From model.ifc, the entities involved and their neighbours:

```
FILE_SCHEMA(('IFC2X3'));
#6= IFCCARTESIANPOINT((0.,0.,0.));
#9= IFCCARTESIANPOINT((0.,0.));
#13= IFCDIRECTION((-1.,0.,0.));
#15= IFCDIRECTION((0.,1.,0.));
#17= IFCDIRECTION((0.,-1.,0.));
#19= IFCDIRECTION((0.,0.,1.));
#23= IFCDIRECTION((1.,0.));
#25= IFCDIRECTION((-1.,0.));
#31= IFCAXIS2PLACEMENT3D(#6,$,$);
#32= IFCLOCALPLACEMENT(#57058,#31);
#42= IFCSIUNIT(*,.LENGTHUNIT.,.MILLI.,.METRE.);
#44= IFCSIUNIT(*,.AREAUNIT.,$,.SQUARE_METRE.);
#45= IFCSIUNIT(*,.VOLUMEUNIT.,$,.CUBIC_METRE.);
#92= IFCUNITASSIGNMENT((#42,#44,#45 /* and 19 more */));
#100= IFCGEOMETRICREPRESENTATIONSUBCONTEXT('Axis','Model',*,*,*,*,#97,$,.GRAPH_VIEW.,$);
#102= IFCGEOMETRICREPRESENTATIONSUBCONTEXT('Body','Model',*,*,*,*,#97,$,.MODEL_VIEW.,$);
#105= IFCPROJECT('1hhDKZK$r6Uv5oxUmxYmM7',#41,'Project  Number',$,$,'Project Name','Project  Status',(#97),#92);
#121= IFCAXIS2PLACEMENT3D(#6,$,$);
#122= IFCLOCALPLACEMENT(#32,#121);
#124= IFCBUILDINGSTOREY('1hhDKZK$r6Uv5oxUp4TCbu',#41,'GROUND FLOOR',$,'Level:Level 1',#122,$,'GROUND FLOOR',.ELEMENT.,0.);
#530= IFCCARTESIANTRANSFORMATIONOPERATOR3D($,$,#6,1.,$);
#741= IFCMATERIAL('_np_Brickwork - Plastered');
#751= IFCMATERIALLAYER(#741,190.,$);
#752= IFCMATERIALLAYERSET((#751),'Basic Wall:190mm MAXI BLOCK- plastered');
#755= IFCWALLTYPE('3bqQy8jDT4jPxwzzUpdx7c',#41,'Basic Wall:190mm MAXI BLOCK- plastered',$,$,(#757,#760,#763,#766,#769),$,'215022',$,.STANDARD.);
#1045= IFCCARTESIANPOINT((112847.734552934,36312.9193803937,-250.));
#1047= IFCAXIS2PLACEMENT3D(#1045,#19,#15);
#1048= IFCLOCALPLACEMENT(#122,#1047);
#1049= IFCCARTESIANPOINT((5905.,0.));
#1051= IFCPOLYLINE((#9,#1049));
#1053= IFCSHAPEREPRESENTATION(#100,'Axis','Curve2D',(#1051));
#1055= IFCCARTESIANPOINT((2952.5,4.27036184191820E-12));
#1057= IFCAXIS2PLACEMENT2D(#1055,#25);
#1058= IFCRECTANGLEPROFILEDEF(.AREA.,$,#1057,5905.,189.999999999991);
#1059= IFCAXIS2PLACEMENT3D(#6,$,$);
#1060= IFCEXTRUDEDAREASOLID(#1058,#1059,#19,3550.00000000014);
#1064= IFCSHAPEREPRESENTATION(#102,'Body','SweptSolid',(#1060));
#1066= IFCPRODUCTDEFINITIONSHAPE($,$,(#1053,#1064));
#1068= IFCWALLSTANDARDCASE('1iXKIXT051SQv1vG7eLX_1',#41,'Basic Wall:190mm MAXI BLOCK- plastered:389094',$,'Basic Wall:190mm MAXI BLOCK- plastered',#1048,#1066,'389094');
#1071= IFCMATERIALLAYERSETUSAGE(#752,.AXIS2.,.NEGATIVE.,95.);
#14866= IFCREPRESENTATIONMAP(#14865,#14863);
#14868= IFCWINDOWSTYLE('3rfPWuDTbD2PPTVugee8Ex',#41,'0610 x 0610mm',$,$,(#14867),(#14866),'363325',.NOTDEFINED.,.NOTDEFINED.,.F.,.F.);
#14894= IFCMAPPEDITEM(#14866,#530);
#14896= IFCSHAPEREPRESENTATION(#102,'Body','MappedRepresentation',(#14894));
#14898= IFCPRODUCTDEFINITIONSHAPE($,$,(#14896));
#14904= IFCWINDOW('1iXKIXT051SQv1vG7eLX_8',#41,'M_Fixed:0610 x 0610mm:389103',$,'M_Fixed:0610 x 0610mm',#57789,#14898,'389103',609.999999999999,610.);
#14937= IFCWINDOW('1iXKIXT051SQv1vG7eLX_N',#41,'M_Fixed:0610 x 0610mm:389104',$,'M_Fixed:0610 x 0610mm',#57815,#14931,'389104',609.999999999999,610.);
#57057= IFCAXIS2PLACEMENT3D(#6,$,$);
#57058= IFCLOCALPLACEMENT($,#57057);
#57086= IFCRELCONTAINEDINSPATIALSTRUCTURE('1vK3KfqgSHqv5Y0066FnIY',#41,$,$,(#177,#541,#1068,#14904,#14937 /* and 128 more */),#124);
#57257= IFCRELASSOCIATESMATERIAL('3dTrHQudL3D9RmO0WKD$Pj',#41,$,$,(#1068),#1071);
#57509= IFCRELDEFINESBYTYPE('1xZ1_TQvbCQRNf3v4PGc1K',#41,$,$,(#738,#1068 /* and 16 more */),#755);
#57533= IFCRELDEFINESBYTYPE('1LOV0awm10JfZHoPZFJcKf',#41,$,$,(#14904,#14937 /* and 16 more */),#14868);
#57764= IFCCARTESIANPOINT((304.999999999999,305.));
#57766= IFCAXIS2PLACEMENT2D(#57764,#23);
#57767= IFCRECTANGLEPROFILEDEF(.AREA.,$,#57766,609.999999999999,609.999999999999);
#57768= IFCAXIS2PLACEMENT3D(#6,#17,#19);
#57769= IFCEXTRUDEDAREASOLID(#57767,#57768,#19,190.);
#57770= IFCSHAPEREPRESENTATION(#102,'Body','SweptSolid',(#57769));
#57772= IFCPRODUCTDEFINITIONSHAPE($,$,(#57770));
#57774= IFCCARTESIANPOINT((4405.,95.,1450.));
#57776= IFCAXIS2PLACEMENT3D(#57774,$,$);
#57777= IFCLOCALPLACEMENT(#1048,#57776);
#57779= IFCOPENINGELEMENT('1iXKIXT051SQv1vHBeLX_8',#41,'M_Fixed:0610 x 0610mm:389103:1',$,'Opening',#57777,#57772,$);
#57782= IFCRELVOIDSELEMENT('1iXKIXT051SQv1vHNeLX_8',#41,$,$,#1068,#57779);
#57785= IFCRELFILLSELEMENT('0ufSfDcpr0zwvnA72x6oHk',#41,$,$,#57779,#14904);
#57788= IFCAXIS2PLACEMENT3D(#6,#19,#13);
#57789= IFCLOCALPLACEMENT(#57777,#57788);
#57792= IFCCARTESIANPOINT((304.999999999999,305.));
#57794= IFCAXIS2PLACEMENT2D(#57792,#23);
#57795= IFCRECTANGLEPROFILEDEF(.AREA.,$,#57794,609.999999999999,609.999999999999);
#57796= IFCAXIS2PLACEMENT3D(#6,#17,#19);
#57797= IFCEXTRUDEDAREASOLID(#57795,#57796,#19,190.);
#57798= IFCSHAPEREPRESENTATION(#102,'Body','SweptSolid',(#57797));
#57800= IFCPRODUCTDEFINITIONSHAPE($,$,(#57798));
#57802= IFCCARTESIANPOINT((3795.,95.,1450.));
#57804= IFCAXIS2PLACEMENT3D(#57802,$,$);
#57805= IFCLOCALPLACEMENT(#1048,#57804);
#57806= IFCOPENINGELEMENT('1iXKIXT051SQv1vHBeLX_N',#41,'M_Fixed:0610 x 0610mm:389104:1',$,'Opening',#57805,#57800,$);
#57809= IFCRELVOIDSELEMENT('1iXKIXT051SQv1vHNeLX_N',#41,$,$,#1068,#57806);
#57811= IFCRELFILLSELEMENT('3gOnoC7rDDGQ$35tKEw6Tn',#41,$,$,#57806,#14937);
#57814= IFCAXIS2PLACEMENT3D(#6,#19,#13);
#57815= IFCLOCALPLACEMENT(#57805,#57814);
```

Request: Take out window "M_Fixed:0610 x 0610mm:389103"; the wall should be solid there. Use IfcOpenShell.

```python
import ifcopenshell
import ifcopenshell.api.feature
import ifcopenshell.api.root
import ifcopenshell.geom
import ifcopenshell.util.shape

model = ifcopenshell.open("model.ifc")
settings = ifcopenshell.geom.settings()


def volume(element):
    """Net volume in cubic metres, openings subtracted."""
    shape = ifcopenshell.geom.create_shape(settings, element)
    return ifcopenshell.util.shape.get_volume(shape.geometry)


window = model.by_guid("1iXKIXT051SQv1vG7eLX_8")
opening = window.FillsVoids[0].RelatingOpeningElement
wall = opening.VoidsElements[0].RelatingBuildingElement
before = volume(wall)

ifcopenshell.api.root.remove_product(model, product=window)
ifcopenshell.api.feature.remove_feature(model, feature=opening)

after = volume(wall)

print(f"wall volume {before:.3f} -> {after:.3f} m3")

model.write("model_edited.ifc")
```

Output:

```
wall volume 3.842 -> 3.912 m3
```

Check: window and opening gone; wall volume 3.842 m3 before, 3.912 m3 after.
